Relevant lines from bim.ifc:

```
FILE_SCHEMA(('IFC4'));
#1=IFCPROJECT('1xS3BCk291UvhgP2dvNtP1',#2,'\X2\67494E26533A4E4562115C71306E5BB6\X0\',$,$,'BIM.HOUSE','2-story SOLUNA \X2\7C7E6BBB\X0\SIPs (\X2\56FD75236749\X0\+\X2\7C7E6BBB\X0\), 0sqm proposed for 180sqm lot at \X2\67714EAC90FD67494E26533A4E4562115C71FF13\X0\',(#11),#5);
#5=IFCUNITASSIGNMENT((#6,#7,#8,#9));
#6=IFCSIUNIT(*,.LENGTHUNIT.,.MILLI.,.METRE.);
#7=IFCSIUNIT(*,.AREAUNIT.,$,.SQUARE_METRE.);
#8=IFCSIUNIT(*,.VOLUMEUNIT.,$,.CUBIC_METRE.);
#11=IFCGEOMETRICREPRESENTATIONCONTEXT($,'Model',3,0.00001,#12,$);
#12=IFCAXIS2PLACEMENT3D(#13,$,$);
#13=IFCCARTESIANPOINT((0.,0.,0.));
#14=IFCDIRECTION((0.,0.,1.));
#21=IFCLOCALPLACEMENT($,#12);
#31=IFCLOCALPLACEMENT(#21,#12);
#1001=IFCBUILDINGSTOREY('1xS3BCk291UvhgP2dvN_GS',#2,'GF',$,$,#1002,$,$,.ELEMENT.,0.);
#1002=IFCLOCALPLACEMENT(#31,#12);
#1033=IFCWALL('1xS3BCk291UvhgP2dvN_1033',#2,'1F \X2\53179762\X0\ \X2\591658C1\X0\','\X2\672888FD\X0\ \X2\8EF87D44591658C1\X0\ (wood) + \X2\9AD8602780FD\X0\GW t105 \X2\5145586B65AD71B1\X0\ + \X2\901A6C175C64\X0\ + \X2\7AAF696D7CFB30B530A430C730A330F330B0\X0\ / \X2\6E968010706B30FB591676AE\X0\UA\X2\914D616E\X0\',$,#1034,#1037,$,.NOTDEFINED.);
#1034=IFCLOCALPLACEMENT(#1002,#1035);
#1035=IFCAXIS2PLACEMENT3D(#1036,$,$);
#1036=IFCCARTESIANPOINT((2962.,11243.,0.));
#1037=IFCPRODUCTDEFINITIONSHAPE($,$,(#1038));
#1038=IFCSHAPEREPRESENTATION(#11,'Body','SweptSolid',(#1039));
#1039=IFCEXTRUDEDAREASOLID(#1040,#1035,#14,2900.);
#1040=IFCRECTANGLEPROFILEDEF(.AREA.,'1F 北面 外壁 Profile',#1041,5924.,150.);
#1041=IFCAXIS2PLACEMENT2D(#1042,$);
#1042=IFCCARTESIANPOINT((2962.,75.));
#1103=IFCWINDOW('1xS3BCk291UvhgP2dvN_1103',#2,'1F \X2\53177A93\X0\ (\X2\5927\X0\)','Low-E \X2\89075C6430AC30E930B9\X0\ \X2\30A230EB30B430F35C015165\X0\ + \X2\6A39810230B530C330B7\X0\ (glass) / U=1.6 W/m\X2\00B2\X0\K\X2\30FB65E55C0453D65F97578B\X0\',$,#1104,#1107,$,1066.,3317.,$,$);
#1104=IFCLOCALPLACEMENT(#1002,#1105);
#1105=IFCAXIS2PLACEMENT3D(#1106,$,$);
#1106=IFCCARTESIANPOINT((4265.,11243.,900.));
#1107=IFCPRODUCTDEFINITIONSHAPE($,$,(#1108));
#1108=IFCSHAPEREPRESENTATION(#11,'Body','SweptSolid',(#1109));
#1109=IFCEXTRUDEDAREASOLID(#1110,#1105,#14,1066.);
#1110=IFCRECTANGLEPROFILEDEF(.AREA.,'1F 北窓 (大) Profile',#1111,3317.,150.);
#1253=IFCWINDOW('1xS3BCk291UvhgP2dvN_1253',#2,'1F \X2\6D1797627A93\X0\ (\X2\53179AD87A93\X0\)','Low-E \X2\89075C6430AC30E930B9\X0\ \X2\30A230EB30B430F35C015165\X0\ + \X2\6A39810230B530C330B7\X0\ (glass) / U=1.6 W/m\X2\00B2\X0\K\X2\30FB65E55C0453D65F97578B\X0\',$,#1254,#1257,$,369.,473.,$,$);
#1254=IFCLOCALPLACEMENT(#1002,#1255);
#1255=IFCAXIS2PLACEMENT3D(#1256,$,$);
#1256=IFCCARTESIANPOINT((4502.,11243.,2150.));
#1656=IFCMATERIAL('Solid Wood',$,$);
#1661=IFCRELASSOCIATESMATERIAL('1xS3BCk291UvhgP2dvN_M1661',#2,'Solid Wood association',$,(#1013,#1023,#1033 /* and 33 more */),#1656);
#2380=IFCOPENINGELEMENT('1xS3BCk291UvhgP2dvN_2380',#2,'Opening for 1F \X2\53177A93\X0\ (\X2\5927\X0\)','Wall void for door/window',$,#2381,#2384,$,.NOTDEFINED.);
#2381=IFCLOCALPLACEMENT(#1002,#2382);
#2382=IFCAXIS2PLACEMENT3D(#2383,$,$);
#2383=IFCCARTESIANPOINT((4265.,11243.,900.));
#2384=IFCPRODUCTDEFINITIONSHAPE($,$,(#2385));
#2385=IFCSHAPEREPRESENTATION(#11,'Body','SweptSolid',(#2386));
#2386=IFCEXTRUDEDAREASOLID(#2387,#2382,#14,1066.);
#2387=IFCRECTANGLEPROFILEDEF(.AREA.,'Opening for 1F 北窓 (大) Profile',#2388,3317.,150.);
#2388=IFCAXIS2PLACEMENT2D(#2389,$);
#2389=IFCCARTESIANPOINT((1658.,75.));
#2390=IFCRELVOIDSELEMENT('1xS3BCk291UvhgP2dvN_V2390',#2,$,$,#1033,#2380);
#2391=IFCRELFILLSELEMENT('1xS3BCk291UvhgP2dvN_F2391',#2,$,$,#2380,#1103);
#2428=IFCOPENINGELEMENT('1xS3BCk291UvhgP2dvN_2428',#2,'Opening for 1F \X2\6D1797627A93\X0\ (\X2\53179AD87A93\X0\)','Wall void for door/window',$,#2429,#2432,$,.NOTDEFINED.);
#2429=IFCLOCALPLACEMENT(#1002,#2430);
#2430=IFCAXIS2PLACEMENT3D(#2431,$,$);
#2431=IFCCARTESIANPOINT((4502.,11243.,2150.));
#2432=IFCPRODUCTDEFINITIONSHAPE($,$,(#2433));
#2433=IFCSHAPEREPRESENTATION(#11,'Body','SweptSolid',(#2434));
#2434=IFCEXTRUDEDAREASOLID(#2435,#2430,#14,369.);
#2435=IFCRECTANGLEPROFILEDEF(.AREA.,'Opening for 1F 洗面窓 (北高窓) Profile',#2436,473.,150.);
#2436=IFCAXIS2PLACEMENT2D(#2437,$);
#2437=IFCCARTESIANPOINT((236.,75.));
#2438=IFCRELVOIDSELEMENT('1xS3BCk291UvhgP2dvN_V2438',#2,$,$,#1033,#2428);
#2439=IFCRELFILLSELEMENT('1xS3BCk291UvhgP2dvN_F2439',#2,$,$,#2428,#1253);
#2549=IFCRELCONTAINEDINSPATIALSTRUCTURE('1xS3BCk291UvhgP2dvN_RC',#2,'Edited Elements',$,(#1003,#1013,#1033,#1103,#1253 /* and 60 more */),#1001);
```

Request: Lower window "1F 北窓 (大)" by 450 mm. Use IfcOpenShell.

```python
import numpy as np
import ifcopenshell
import ifcopenshell.api.geometry
import ifcopenshell.util.placement
import ifcopenshell.util.unit

model = ifcopenshell.open("bim.ifc")
unit_scale = ifcopenshell.util.unit.calculate_unit_scale(model)

window = model.by_guid("1xS3BCk291UvhgP2dvN_1103")
opening = window.FillsVoids[0].RelatingOpeningElement
dz = -0.45 / unit_scale

shift = np.array([0.0, 0.0, dz])
# The window is not placed relative to its opening, so move both.
for product in (opening, window):
    matrix = ifcopenshell.util.placement.get_local_placement(product.ObjectPlacement)
    matrix[:3, 3] += shift
    ifcopenshell.api.geometry.edit_object_placement(model, product=product, matrix=matrix, is_si=False)

print(f"moved by {dz * unit_scale:+.3f} m")

model.write("bim_edited.ifc")
```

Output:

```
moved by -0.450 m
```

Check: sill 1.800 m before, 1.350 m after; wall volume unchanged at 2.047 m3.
